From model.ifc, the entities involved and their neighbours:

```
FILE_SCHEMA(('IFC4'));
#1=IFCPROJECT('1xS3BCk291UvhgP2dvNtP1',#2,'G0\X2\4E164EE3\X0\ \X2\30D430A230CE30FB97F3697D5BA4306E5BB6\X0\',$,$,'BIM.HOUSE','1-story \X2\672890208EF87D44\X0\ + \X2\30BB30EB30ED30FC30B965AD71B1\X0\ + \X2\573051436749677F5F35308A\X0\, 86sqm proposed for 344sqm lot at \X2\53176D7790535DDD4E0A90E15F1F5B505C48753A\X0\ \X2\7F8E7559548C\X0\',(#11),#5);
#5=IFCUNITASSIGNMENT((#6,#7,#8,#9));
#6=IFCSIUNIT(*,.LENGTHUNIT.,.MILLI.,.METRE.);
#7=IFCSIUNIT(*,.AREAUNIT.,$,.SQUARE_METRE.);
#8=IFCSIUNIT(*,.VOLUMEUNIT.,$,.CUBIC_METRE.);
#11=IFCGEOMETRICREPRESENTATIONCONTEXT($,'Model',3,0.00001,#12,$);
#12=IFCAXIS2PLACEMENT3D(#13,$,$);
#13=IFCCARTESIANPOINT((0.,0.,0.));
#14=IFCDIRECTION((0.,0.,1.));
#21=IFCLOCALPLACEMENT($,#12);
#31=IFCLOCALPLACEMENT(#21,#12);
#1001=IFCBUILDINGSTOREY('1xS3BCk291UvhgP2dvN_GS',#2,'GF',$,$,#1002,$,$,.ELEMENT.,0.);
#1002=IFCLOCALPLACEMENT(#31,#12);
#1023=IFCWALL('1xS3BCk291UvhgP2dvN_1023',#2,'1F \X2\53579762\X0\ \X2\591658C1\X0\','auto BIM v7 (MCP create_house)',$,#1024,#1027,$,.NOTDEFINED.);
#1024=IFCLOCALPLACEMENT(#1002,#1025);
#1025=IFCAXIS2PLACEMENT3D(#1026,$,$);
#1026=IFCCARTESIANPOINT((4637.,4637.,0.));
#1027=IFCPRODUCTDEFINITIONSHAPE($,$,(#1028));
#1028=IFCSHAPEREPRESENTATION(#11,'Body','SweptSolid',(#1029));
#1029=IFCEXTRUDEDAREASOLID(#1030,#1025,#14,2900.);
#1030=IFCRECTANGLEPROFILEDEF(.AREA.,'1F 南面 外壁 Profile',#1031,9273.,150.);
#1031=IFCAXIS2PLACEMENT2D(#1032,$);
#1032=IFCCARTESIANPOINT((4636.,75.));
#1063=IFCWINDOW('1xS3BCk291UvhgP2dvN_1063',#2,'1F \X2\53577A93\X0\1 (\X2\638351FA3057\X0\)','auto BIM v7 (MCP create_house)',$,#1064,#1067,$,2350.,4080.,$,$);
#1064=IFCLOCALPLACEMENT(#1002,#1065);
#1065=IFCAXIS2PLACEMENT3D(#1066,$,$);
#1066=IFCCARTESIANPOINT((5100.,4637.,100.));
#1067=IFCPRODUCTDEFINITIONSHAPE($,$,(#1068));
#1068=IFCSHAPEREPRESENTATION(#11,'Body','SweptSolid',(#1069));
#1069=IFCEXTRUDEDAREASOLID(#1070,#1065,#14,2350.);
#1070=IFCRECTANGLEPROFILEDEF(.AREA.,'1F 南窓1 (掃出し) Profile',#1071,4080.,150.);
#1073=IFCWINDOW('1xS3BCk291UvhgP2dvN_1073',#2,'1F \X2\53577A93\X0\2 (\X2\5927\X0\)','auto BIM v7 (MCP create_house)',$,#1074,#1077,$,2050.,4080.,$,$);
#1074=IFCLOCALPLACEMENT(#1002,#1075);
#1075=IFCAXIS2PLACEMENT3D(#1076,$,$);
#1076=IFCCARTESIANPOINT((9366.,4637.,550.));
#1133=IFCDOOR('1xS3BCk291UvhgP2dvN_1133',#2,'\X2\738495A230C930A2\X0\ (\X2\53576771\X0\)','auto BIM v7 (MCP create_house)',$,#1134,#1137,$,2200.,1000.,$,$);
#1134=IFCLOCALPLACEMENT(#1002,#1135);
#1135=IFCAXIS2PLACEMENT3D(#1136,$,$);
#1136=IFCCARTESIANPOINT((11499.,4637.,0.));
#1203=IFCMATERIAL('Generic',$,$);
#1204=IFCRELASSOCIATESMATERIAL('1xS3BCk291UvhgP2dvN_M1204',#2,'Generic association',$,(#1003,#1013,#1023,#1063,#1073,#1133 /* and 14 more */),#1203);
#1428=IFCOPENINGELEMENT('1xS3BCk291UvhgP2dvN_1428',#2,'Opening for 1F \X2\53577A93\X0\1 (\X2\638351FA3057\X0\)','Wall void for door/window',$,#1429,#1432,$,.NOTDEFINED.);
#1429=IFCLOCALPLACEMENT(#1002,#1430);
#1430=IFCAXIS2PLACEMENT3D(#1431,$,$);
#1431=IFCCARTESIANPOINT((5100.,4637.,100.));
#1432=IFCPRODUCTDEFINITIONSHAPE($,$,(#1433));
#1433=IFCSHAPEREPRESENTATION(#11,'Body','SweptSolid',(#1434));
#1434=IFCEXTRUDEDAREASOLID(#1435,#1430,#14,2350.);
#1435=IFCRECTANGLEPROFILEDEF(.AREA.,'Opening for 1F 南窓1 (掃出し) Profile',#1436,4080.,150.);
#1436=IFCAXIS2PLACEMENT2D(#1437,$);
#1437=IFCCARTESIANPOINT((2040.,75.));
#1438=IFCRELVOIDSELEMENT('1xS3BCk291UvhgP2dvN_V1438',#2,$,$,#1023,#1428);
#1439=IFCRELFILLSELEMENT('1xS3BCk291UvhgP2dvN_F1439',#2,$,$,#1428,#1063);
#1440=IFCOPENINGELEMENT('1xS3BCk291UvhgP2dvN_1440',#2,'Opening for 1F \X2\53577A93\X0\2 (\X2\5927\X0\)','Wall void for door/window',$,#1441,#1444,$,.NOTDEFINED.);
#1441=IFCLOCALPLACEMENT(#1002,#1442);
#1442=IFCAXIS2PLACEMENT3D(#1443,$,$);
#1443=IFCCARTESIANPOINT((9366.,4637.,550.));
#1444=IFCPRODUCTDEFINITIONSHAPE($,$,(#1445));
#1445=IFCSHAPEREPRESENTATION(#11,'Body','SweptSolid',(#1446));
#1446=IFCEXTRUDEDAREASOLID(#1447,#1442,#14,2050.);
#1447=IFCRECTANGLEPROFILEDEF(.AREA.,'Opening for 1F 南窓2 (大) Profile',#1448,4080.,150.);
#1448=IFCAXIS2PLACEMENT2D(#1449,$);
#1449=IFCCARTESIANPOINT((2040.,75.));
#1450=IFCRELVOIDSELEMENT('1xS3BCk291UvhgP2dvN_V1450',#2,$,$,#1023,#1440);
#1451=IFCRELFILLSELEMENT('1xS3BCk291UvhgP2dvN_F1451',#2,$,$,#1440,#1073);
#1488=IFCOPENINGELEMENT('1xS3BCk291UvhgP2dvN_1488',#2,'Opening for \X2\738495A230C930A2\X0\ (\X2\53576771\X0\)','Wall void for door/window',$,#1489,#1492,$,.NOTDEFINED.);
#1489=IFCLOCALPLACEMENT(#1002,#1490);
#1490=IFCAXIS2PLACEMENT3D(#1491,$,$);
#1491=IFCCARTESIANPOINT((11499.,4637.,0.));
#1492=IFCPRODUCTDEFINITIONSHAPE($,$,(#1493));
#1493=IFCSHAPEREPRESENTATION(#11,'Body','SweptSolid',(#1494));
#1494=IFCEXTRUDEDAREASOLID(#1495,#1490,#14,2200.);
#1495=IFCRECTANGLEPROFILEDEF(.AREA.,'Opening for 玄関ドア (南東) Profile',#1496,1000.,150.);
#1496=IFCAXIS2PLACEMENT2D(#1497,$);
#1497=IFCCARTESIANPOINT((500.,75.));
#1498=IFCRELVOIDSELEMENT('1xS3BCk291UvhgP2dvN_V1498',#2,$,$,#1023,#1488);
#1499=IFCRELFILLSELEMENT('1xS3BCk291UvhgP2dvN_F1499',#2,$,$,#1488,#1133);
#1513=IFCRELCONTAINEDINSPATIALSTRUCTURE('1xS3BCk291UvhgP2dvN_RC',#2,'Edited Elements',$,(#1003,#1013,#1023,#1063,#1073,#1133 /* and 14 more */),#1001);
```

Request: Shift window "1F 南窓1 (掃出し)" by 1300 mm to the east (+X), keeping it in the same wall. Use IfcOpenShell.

```python
import ifcopenshell
import ifcopenshell.api.geometry
import ifcopenshell.util.placement

model = ifcopenshell.open("model.ifc")

window = model.by_guid("1xS3BCk291UvhgP2dvN_1063")
opening = window.FillsVoids[0].RelatingOpeningElement
wall = opening.VoidsElements[0].RelatingBuildingElement

wall_matrix = ifcopenshell.util.placement.get_local_placement(wall.ObjectPlacement)
shift = wall_matrix[:3, 0] * 1300.0
before = ifcopenshell.util.placement.get_local_placement(window.ObjectPlacement)[:3, 3].copy()

# The window is not placed relative to its opening, so move both.
for product in (opening, window):
    matrix = ifcopenshell.util.placement.get_local_placement(product.ObjectPlacement)
    matrix[:3, 3] += shift
    ifcopenshell.api.geometry.edit_object_placement(model, product=product, matrix=matrix, is_si=False)

after = ifcopenshell.util.placement.get_local_placement(window.ObjectPlacement)[:3, 3]
print("window moved by", (after - before).round(3) + 0.0)

model.write("model_updated.ifc")
```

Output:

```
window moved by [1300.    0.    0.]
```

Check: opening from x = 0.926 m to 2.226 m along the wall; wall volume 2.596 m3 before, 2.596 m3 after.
